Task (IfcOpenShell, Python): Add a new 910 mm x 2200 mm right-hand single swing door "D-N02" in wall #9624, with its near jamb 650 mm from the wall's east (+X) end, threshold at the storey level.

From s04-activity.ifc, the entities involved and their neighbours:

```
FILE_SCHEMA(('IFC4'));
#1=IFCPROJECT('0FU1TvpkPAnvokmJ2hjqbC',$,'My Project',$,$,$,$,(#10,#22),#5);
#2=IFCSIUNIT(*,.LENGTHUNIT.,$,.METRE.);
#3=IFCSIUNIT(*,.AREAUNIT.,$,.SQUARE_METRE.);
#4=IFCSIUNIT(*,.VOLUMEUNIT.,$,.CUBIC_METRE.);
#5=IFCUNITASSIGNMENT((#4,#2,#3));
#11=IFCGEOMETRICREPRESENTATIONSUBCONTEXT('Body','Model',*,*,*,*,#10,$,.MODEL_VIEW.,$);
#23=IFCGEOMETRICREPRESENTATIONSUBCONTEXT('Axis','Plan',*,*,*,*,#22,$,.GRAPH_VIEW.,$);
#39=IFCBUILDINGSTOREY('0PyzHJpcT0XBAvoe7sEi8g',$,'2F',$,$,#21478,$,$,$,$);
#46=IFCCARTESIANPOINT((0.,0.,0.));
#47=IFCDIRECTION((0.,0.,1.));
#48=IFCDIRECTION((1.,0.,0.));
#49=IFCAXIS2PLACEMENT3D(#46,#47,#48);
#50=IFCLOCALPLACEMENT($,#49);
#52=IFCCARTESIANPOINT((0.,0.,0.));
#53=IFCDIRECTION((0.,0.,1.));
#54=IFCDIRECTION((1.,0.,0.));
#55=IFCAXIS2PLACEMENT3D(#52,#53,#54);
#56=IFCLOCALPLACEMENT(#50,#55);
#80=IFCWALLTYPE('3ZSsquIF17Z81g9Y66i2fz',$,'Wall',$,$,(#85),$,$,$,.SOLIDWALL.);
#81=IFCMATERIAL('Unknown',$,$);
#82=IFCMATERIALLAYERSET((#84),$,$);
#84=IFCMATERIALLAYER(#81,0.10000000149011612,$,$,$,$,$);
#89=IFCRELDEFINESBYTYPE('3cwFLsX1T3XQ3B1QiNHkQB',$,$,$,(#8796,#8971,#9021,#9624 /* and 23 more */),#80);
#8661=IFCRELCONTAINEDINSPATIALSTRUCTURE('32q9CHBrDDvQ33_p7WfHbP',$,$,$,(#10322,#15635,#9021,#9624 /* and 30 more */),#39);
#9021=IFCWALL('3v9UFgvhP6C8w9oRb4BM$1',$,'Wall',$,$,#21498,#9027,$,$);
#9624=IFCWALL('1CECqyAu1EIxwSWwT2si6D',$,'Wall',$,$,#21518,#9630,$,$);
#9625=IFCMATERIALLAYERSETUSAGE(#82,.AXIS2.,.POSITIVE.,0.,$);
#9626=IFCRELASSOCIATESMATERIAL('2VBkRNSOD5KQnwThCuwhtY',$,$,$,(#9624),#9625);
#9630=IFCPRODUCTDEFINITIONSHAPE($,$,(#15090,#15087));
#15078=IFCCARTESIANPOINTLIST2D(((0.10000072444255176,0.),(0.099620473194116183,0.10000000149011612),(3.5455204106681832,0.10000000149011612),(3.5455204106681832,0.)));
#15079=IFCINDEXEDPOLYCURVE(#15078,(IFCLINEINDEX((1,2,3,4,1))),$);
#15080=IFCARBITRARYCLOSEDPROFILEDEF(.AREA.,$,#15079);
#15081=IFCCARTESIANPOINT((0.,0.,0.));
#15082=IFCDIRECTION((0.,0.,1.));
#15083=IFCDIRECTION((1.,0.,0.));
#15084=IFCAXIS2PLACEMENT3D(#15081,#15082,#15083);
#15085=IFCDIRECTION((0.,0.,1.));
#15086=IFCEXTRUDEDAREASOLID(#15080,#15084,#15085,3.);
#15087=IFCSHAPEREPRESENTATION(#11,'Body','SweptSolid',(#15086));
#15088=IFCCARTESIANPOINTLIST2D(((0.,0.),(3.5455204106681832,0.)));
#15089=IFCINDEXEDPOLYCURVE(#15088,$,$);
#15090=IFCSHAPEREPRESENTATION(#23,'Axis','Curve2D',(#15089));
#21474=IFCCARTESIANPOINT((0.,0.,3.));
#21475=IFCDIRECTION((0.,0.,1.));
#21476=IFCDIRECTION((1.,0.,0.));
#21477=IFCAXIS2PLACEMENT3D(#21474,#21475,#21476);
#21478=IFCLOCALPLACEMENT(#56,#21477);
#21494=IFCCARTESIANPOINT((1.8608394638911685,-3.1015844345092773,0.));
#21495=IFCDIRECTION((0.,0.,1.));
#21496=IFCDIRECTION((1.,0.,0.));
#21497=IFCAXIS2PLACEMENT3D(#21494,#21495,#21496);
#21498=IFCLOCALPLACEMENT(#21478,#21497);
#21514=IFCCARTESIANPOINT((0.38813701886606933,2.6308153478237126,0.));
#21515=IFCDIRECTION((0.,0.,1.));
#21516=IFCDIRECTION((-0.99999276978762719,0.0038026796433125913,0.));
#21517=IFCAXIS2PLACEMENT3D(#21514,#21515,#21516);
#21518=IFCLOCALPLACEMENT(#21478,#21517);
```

```python
import numpy as np
import ifcopenshell
import ifcopenshell.api.feature
import ifcopenshell.api.geometry
import ifcopenshell.api.root
import ifcopenshell.api.spatial
import ifcopenshell.geom
import ifcopenshell.util.element
import ifcopenshell.util.placement
import ifcopenshell.util.representation
import ifcopenshell.util.shape
import ifcopenshell.util.unit

model = ifcopenshell.open("s04-activity.ifc")
unit_scale = ifcopenshell.util.unit.calculate_unit_scale(model)
settings = ifcopenshell.geom.settings()


def volume(element):
    """Net volume in cubic metres, openings subtracted."""
    shape = ifcopenshell.geom.create_shape(settings, element)
    return ifcopenshell.util.shape.get_volume(shape.geometry)


wall = model.by_guid("1CECqyAu1EIxwSWwT2si6D")
storey = ifcopenshell.util.element.get_container(wall, ifc_class="IfcBuildingStorey")
context = ifcopenshell.util.representation.get_context(model, "Model", "Body", "MODEL_VIEW")
before = volume(wall)

width, height, from_end, sill = 0.91, 2.2, 0.65, 0.0  # metres

# The wall runs along its own X axis, and the end named is its -X end.
wall_shape = ifcopenshell.geom.create_shape(settings, wall)
x, y, z = ifcopenshell.util.shape.get_vertices(wall_shape.geometry).T
start = x.min() + from_end
face, thickness = float(y.min()), float(y.max() - y.min())
wall_matrix = ifcopenshell.util.placement.get_local_placement(wall.ObjectPlacement)
level = ifcopenshell.util.placement.get_local_placement(storey.ObjectPlacement)[2, 3]


def in_wall(x, y):
    """Placement at x, y metres in the wall's axes, at sill height."""
    matrix = wall_matrix.copy()
    matrix[:, 3] = wall_matrix @ np.array([x / unit_scale, y / unit_scale, 0.0, 1.0])
    matrix[2, 3] = level + sill / unit_scale
    return matrix


# Opening: a box that overshoots both wall faces by 50 mm.
opening = ifcopenshell.api.root.create_entity(model, ifc_class="IfcOpeningElement", predefined_type="OPENING")
box = ifcopenshell.api.geometry.add_wall_representation(
    model, context=context, length=width, height=height, thickness=thickness + 0.1
)
ifcopenshell.api.geometry.assign_representation(model, product=opening, representation=box)
ifcopenshell.api.geometry.edit_object_placement(model, product=opening, matrix=in_wall(start, face - 0.05), is_si=False)
ifcopenshell.api.feature.add_feature(model, feature=opening, element=wall)

door = ifcopenshell.api.root.create_entity(model, ifc_class="IfcDoor", name="D-N02", predefined_type="DOOR")
door.OverallWidth, door.OverallHeight = width / unit_scale, height / unit_scale
door.OperationType = "SINGLE_SWING_RIGHT"
body = ifcopenshell.api.geometry.add_door_representation(
    model,
    context=context,
    overall_width=door.OverallWidth,
    overall_height=door.OverallHeight,
    operation_type="SINGLE_SWING_RIGHT",
    lining_properties={"LiningDepth": thickness / unit_scale, "ThresholdDepth": thickness / unit_scale},
)
ifcopenshell.api.geometry.assign_representation(model, product=door, representation=body)
ifcopenshell.api.spatial.assign_container(model, products=[door], relating_structure=storey)
ifcopenshell.api.feature.add_filling(model, opening=opening, element=door)

# The lining spans the wall, so the door starts at the wall face.
ifcopenshell.api.geometry.edit_object_placement(model, product=door, matrix=in_wall(start, face), is_si=False)

after = volume(wall)

print(f"wall volume {before:.3f} -> {after:.3f} m3")

model.write("s04-activity-out.ifc")
```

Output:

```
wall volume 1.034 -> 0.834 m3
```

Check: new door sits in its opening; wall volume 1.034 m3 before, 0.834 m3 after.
